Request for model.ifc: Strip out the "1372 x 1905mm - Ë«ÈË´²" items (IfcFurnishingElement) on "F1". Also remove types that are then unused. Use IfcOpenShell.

First a look at what the model holds.

```python
import ifcopenshell
import ifcopenshell.util.element

model = ifcopenshell.open("model.ifc")
print(model.schema)
storey = next(s for s in model.by_type("IfcBuildingStorey") if s.Name == "F1")
furniture = [e for e in ifcopenshell.util.element.get_decomposition(storey) if e.is_a("IfcFurnishingElement")]
seen = {}
for e in furniture:
    element_type = ifcopenshell.util.element.get_type(e)
    name = element_type.Name if element_type not in (None, e) else None
    seen[name] = seen.get(name, 0) + 1
for name, count in sorted(seen.items(), key=str):
    print(count, "x", name)
```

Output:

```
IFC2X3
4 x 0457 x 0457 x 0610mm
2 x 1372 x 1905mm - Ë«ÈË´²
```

```python
import ifcopenshell
import ifcopenshell.api.root
import ifcopenshell.util.element

model = ifcopenshell.open("model.ifc")

storey = next(s for s in model.by_type("IfcBuildingStorey") if s.Name == "F1")
furniture = [e for e in ifcopenshell.util.element.get_decomposition(storey) if e.is_a("IfcFurnishingElement")]
targets = [e for e in furniture if (t := ifcopenshell.util.element.get_type(e)) not in (None, e) and t.Name == "1372 x 1905mm - Ë«ÈË´²"]
types = {ifcopenshell.util.element.get_type(e) for e in targets} - {None, *targets}

for e in targets:
    ifcopenshell.api.root.remove_product(model, product=e)
print(len(targets), "removed")

unused = [t for t in types if not ifcopenshell.util.element.get_types(t)]
for t in unused:
    ifcopenshell.api.root.remove_product(model, product=t)
print(len(unused), "unused types removed")

model.write("model_edited.ifc")
```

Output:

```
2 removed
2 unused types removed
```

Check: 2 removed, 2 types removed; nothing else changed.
